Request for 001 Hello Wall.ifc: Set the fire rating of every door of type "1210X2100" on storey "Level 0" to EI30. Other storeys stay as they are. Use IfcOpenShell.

First a look at what the model holds.

```python
import ifcopenshell
import ifcopenshell.util.element

model = ifcopenshell.open("001 Hello Wall.ifc")
print(model.schema)
storey = next(s for s in model.by_type("IfcBuildingStorey") if s.Name == "Level 0")
doors = [e for e in ifcopenshell.util.element.get_decomposition(storey) if e.is_a("IfcDoor")]
seen = {}
for e in doors:
    element_type = ifcopenshell.util.element.get_type(e)
    key = (element_type.Name if element_type != e and element_type else None, ifcopenshell.util.element.get_pset(e, "Pset_DoorCommon", "FireRating"))
    seen[key] = seen.get(key, 0) + 1
for (name, value), count in sorted(seen.items(), key=str):
    print(count, "x", name, "|", value)
```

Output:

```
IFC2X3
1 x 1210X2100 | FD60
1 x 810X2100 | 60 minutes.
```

```python
import ifcopenshell
import ifcopenshell.api.pset
import ifcopenshell.util.element

model = ifcopenshell.open("001 Hello Wall.ifc")

storey = next(s for s in model.by_type("IfcBuildingStorey") if s.Name == "Level 0")
doors = [e for e in ifcopenshell.util.element.get_decomposition(storey) if e.is_a("IfcDoor")]

count = 0
for e in doors:
    element_type = ifcopenshell.util.element.get_type(e)
    if element_type in (None, e) or element_type.Name != "1210X2100":
        continue
    # add_pset returns the element's existing set when there is one.
    pset = ifcopenshell.api.pset.add_pset(model, product=e, name="Pset_DoorCommon")
    ifcopenshell.api.pset.edit_pset(model, pset=pset, properties={"FireRating": "EI30"})
    count += 1

print(count, "doors updated")

model.write("001 Hello Wall_v2.ifc")
```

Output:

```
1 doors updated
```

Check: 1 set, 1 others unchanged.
